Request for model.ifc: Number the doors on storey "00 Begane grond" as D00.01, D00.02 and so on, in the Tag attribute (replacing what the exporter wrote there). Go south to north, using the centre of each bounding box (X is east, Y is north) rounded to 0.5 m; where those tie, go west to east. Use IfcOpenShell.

First a look at what the model holds.

```python
import ifcopenshell
import ifcopenshell.util.element
import ifcopenshell.util.placement

model = ifcopenshell.open("model.ifc")
print(model.schema)
storey = next(s for s in model.by_type("IfcBuildingStorey") if s.Name == "00 Begane grond")
doors = [e for e in ifcopenshell.util.element.get_decomposition(storey) if e.is_a("IfcDoor")]
for e in sorted(doors, key=lambda e: e.id()):
    origin = ifcopenshell.util.placement.get_local_placement(e.ObjectPlacement)[:3, 3]
    print(e.id(), e.Tag, e.Name, origin.round(2) + 0.0, sep=" | ")
```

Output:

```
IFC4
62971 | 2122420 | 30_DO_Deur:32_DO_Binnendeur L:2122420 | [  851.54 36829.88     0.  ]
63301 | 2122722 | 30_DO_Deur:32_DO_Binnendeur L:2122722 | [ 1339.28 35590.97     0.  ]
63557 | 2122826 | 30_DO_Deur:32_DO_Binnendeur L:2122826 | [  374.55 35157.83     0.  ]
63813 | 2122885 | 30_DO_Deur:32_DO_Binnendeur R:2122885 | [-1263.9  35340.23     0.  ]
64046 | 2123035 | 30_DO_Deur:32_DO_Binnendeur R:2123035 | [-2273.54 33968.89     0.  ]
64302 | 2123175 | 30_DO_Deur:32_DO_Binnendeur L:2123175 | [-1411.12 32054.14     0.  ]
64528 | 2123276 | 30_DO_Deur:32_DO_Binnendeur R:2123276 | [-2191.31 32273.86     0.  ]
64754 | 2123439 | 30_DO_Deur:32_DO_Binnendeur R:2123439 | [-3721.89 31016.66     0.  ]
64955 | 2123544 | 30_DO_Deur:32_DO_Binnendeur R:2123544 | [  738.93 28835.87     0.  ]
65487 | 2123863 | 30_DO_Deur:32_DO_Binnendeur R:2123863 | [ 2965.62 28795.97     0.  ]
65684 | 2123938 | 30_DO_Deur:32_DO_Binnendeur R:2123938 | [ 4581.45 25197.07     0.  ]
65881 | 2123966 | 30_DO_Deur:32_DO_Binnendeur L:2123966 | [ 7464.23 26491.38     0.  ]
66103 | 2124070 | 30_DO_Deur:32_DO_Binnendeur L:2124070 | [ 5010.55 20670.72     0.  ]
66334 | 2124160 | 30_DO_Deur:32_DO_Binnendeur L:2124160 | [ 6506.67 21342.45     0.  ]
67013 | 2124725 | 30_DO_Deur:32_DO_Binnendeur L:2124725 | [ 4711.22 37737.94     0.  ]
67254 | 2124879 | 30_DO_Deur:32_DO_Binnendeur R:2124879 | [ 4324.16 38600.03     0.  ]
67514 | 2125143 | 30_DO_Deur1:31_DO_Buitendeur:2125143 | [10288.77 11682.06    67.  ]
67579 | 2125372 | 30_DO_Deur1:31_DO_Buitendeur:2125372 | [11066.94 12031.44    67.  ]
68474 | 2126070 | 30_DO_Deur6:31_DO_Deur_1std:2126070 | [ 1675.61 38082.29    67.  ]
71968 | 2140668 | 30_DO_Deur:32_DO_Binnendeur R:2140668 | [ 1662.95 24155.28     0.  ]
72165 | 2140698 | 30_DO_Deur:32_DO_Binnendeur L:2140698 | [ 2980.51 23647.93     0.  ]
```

```python
import ifcopenshell
import ifcopenshell.geom
import ifcopenshell.util.element
import ifcopenshell.util.shape

model = ifcopenshell.open("model.ifc")
settings = ifcopenshell.geom.settings()
settings.set("use-world-coords", True)


def centre(element):
    shape = ifcopenshell.geom.create_shape(settings, element)
    return ifcopenshell.util.shape.get_bbox_centroid(shape.geometry)


storey = next(s for s in model.by_type("IfcBuildingStorey") if s.Name == "00 Begane grond")
doors = [e for e in ifcopenshell.util.element.get_decomposition(storey) if e.is_a("IfcDoor")]

# Insertion points can sit at a corner or the storey origin, so sort by the geometry (in metres).
centres = {e: centre(e) for e in doors}
doors.sort(key=lambda e: (round(centres[e][1] / 0.5), centres[e][0]))

for i, e in enumerate(doors, start=1):
    number = f"D00.{i:02d}"
    e.Tag = number
    print(e.id(), number)

model.write("model_rev.ifc")
```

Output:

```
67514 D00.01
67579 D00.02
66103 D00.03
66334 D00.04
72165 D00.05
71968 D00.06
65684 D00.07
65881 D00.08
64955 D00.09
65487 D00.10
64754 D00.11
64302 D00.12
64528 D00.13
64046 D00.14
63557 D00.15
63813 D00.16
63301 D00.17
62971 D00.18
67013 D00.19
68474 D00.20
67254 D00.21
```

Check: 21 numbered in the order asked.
